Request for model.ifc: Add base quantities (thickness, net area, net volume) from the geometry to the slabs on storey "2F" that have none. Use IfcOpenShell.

First a look at what the model holds.

```python
import ifcopenshell
import ifcopenshell.util.element
import ifcopenshell.util.unit

model = ifcopenshell.open("model.ifc")
print(model.schema)
for unit_type in ("LENGTHUNIT", "AREAUNIT", "VOLUMEUNIT"):
    print(unit_type, ifcopenshell.util.unit.calculate_unit_scale(model, unit_type))
storey = next(s for s in model.by_type("IfcBuildingStorey") if s.Name == "2F")
slabs = [e for e in ifcopenshell.util.element.get_decomposition(storey) if e.is_a("IfcSlab")]
for e in sorted(slabs, key=lambda e: e.id()):
    print(e.id(), e.is_a(), e.Name, list(ifcopenshell.util.element.get_psets(e, qtos_only=True)), sep=" | ")
```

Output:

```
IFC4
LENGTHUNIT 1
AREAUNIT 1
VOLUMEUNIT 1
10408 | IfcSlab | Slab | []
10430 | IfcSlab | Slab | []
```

```python
import ifcopenshell
import ifcopenshell.api.pset
import ifcopenshell.geom
import ifcopenshell.util.element
import ifcopenshell.util.shape
import ifcopenshell.util.unit

model = ifcopenshell.open("model.ifc")
unit_scale = ifcopenshell.util.unit.calculate_unit_scale(model)
area_scale = ifcopenshell.util.unit.calculate_unit_scale(model, "AREAUNIT")
volume_scale = ifcopenshell.util.unit.calculate_unit_scale(model, "VOLUMEUNIT")
settings = ifcopenshell.geom.settings()

storey = next(s for s in model.by_type("IfcBuildingStorey") if s.Name == "2F")
slabs = [e for e in ifcopenshell.util.element.get_decomposition(storey) if e.is_a("IfcSlab")]

for e in sorted(slabs, key=lambda e: e.id()):
    if ifcopenshell.util.element.get_psets(e, qtos_only=True, should_inherit=False):
        continue
    # Geometry comes back in metres, in the element's own axes.
    shape = ifcopenshell.geom.create_shape(settings, e)
    values = {
        "Width": ifcopenshell.util.shape.get_z(shape.geometry) / unit_scale,
        "NetArea": ifcopenshell.util.shape.get_footprint_area(shape.geometry) / area_scale,
        "NetVolume": ifcopenshell.util.shape.get_volume(shape.geometry) / volume_scale,
    }
    qto = ifcopenshell.api.pset.add_qto(model, product=e, name="Qto_SlabBaseQuantities")
    ifcopenshell.api.pset.edit_qto(model, qto=qto, properties=values)
    print(e.id(), {k: round(v, 3) for k, v in values.items()})

model.write("model_v2.ifc")
```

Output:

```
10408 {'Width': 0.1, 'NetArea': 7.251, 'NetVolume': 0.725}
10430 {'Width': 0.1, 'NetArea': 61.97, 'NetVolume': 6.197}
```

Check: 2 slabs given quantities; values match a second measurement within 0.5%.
